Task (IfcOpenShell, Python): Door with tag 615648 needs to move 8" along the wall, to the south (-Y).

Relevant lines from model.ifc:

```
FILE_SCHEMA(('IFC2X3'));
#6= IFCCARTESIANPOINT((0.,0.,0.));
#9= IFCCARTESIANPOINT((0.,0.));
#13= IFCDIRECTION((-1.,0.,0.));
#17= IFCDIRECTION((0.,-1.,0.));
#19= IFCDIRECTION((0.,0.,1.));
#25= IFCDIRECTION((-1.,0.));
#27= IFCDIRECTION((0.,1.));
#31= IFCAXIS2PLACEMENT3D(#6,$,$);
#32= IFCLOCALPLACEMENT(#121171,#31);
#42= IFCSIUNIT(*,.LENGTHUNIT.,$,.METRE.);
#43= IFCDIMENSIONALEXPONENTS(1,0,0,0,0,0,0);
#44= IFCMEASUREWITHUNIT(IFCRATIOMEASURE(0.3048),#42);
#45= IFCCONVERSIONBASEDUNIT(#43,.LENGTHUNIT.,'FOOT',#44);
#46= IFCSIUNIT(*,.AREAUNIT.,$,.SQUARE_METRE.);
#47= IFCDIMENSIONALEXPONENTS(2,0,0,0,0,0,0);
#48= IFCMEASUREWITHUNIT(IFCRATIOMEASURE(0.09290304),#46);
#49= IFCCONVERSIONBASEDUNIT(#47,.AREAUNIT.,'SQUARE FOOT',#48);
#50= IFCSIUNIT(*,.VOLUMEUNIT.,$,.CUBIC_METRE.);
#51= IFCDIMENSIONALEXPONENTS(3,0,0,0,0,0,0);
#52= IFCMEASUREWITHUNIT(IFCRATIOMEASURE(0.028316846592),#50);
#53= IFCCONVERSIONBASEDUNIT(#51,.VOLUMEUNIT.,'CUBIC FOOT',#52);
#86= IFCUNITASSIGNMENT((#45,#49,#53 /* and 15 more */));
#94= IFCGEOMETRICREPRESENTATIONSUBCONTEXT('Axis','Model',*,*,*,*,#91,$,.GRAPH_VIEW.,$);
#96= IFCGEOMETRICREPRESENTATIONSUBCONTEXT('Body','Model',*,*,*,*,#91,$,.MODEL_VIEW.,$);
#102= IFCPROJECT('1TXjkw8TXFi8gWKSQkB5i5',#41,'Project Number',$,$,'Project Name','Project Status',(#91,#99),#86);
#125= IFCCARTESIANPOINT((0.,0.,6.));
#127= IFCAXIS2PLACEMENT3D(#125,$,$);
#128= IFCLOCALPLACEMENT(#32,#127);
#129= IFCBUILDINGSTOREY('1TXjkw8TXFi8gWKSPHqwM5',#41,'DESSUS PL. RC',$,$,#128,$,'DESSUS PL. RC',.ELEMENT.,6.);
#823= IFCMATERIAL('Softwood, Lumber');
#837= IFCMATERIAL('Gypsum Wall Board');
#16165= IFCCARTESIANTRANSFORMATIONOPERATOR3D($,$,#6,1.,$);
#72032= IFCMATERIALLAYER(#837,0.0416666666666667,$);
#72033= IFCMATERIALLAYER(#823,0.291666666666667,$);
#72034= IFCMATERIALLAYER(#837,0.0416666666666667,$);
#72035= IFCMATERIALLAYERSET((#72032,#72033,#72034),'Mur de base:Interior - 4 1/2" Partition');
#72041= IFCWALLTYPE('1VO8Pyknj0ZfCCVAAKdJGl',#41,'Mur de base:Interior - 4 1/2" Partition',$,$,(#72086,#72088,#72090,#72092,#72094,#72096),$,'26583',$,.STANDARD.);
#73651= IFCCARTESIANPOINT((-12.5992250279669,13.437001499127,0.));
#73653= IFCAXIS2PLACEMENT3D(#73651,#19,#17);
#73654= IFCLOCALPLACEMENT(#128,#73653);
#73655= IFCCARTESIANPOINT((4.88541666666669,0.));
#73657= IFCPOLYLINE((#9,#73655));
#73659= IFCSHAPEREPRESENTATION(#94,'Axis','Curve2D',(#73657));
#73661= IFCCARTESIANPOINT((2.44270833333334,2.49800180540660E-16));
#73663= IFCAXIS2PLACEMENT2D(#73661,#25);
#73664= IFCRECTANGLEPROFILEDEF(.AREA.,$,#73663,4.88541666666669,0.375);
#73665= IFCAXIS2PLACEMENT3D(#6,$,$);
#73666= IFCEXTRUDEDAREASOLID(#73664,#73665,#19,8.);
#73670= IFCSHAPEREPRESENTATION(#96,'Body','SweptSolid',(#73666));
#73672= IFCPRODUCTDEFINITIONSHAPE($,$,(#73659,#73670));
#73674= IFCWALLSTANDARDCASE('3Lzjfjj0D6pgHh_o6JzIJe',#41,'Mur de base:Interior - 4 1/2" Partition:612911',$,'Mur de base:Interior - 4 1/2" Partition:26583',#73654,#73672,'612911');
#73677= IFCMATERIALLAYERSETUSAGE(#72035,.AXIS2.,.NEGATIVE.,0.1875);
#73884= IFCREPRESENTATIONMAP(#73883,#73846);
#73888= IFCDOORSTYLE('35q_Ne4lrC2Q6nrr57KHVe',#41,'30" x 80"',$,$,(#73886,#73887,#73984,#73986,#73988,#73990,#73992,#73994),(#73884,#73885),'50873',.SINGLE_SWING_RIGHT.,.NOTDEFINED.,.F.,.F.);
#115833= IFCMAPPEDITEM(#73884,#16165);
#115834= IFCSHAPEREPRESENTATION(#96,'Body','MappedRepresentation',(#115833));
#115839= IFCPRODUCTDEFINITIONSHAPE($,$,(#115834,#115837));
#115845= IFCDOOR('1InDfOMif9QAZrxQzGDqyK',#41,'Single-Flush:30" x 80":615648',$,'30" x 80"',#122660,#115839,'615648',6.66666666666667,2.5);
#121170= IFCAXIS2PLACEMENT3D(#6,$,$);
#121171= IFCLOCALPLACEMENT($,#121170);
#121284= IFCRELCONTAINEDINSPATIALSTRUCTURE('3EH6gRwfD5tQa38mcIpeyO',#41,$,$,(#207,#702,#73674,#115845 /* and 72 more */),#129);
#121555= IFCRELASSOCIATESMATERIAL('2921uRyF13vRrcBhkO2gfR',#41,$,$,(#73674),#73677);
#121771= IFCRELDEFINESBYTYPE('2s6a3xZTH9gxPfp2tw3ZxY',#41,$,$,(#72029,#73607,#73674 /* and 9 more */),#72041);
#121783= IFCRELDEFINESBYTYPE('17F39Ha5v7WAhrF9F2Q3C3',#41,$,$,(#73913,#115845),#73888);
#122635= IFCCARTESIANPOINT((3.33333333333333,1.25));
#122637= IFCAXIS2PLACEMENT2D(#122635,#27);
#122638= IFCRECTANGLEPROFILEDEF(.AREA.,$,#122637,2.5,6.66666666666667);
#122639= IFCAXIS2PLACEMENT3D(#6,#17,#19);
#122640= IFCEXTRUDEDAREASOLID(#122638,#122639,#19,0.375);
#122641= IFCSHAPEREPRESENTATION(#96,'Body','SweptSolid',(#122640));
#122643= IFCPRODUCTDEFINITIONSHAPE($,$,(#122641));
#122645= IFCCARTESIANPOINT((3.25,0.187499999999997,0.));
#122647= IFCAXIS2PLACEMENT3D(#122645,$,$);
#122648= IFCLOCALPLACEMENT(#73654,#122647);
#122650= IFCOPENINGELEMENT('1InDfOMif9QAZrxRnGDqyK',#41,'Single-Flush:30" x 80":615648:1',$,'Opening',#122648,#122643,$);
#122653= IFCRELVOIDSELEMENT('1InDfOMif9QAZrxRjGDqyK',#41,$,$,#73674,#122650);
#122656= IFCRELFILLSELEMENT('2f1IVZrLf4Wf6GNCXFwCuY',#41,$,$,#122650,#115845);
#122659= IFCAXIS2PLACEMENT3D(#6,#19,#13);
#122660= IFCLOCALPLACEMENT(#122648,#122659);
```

```python
import ifcopenshell
import ifcopenshell.api.geometry
import ifcopenshell.util.placement
import ifcopenshell.util.unit

model = ifcopenshell.open("model.ifc")
unit_scale = ifcopenshell.util.unit.calculate_unit_scale(model)

door = model.by_id(115845)
opening = door.FillsVoids[0].RelatingOpeningElement
wall = opening.VoidsElements[0].RelatingBuildingElement

wall_matrix = ifcopenshell.util.placement.get_local_placement(wall.ObjectPlacement)
shift = wall_matrix[:3, 0] * 8 * 0.0254 / unit_scale
before = ifcopenshell.util.placement.get_local_placement(door.ObjectPlacement)[:3, 3].copy()

# The door is placed relative to its opening, so it follows when the opening moves.
matrix = ifcopenshell.util.placement.get_local_placement(opening.ObjectPlacement)
matrix[:3, 3] += shift
ifcopenshell.api.geometry.edit_object_placement(
    model, product=opening, matrix=matrix, is_si=False, should_transform_children=True
)

after = ifcopenshell.util.placement.get_local_placement(door.ObjectPlacement)[:3, 3]
print("door moved by", (after - before).round(3) + 0.0)

model.write("model_v2.ifc")
```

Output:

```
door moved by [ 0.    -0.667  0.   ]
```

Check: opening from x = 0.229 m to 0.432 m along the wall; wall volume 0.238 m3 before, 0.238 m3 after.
